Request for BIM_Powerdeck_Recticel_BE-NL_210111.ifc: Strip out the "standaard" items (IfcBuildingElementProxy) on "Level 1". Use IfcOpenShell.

First a look at what the model holds.

```python
import ifcopenshell
import ifcopenshell.util.element

model = ifcopenshell.open("BIM_Powerdeck_Recticel_BE-NL_210111.ifc")
print(model.schema)
storey = next(s for s in model.by_type("IfcBuildingStorey") if s.Name == "Level 1")
proxies = [e for e in ifcopenshell.util.element.get_decomposition(storey) if e.is_a("IfcBuildingElementProxy")]
seen = {}
for e in proxies:
    element_type = ifcopenshell.util.element.get_type(e)
    name = element_type.Name if element_type not in (None, e) else None
    seen[name] = seen.get(name, 0) + 1
for name, count in sorted(seen.items(), key=str):
    print(count, "x", name)
```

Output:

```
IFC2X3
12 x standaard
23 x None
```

```python
import ifcopenshell
import ifcopenshell.api.root
import ifcopenshell.util.element

model = ifcopenshell.open("BIM_Powerdeck_Recticel_BE-NL_210111.ifc")

storey = next(s for s in model.by_type("IfcBuildingStorey") if s.Name == "Level 1")
proxies = [e for e in ifcopenshell.util.element.get_decomposition(storey) if e.is_a("IfcBuildingElementProxy")]
targets = [e for e in proxies if (t := ifcopenshell.util.element.get_type(e)) not in (None, e) and t.Name == "standaard"]

for e in targets:
    ifcopenshell.api.root.remove_product(model, product=e)
print(len(targets), "removed")

model.write("BIM_Powerdeck_Recticel_BE-NL_210111-out.ifc")
```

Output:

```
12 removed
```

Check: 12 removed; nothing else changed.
